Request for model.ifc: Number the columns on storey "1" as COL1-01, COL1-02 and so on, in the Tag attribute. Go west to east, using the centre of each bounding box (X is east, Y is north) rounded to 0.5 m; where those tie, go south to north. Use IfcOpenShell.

First a look at what the model holds.

```python
import ifcopenshell
import ifcopenshell.util.element
import ifcopenshell.util.placement

model = ifcopenshell.open("model.ifc")
print(model.schema)
storey = next(s for s in model.by_type("IfcBuildingStorey") if s.Name == "1")
columns = [e for e in ifcopenshell.util.element.get_decomposition(storey) if e.is_a("IfcColumn")]
for e in sorted(columns, key=lambda e: e.id()):
    origin = ifcopenshell.util.placement.get_local_placement(e.ObjectPlacement)[:3, 3]
    print(e.id(), e.Tag, e.Name, origin.round(2) + 0.0, sep=" | ")
```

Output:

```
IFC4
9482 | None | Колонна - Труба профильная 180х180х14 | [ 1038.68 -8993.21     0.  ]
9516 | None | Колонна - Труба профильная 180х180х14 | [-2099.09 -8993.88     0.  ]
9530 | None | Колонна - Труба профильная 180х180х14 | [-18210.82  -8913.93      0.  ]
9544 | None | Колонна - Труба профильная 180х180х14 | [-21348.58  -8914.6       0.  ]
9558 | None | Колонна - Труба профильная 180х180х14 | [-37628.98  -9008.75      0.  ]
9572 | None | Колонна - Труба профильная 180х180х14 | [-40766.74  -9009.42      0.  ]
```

```python
import ifcopenshell
import ifcopenshell.geom
import ifcopenshell.util.element
import ifcopenshell.util.shape

model = ifcopenshell.open("model.ifc")
settings = ifcopenshell.geom.settings()
settings.set("use-world-coords", True)


def centre(element):
    shape = ifcopenshell.geom.create_shape(settings, element)
    return ifcopenshell.util.shape.get_bbox_centroid(shape.geometry)


storey = next(s for s in model.by_type("IfcBuildingStorey") if s.Name == "1")
columns = [e for e in ifcopenshell.util.element.get_decomposition(storey) if e.is_a("IfcColumn")]

# Insertion points can sit at a corner or the storey origin, so sort by the geometry (in metres).
centres = {e: centre(e) for e in columns}
columns.sort(key=lambda e: (round(centres[e][0] / 0.5), centres[e][1]))

for i, e in enumerate(columns, start=1):
    number = f"COL1-{i:02d}"
    e.Tag = number
    print(e.id(), number)

model.write("model-out.ifc")
```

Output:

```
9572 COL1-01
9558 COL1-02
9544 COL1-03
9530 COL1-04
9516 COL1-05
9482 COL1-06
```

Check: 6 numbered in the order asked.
